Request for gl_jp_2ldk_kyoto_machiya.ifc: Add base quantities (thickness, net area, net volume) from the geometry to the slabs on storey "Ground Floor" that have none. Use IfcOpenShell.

First a look at what the model holds.

```python
import ifcopenshell
import ifcopenshell.util.element
import ifcopenshell.util.unit

model = ifcopenshell.open("gl_jp_2ldk_kyoto_machiya.ifc")
print(model.schema)
for unit_type in ("LENGTHUNIT", "AREAUNIT", "VOLUMEUNIT"):
    print(unit_type, ifcopenshell.util.unit.calculate_unit_scale(model, unit_type))
storey = next(s for s in model.by_type("IfcBuildingStorey") if s.Name == "Ground Floor")
slabs = [e for e in ifcopenshell.util.element.get_decomposition(storey) if e.is_a("IfcSlab")]
for e in sorted(slabs, key=lambda e: e.id()):
    print(e.id(), e.is_a(), e.Name, list(ifcopenshell.util.element.get_psets(e, qtos_only=True)), sep=" | ")
```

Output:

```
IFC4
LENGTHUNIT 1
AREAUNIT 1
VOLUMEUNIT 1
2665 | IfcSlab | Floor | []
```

```python
import ifcopenshell
import ifcopenshell.api.pset
import ifcopenshell.geom
import ifcopenshell.util.element
import ifcopenshell.util.shape
import ifcopenshell.util.unit

model = ifcopenshell.open("gl_jp_2ldk_kyoto_machiya.ifc")
unit_scale = ifcopenshell.util.unit.calculate_unit_scale(model)
area_scale = ifcopenshell.util.unit.calculate_unit_scale(model, "AREAUNIT")
volume_scale = ifcopenshell.util.unit.calculate_unit_scale(model, "VOLUMEUNIT")
settings = ifcopenshell.geom.settings()

storey = next(s for s in model.by_type("IfcBuildingStorey") if s.Name == "Ground Floor")
slabs = [e for e in ifcopenshell.util.element.get_decomposition(storey) if e.is_a("IfcSlab")]

for e in sorted(slabs, key=lambda e: e.id()):
    if ifcopenshell.util.element.get_psets(e, qtos_only=True, should_inherit=False):
        continue
    # Geometry comes back in metres, in the element's own axes.
    shape = ifcopenshell.geom.create_shape(settings, e)
    values = {
        "Width": ifcopenshell.util.shape.get_z(shape.geometry) / unit_scale,
        "NetArea": ifcopenshell.util.shape.get_footprint_area(shape.geometry) / area_scale,
        "NetVolume": ifcopenshell.util.shape.get_volume(shape.geometry) / volume_scale,
    }
    qto = ifcopenshell.api.pset.add_qto(model, product=e, name="Qto_SlabBaseQuantities")
    ifcopenshell.api.pset.edit_qto(model, qto=qto, properties=values)
    print(e.id(), {k: round(v, 3) for k, v in values.items()})

model.write("gl_jp_2ldk_kyoto_machiya_v2.ifc")
```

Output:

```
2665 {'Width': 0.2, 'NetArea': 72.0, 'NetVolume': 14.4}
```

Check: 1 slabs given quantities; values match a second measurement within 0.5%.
